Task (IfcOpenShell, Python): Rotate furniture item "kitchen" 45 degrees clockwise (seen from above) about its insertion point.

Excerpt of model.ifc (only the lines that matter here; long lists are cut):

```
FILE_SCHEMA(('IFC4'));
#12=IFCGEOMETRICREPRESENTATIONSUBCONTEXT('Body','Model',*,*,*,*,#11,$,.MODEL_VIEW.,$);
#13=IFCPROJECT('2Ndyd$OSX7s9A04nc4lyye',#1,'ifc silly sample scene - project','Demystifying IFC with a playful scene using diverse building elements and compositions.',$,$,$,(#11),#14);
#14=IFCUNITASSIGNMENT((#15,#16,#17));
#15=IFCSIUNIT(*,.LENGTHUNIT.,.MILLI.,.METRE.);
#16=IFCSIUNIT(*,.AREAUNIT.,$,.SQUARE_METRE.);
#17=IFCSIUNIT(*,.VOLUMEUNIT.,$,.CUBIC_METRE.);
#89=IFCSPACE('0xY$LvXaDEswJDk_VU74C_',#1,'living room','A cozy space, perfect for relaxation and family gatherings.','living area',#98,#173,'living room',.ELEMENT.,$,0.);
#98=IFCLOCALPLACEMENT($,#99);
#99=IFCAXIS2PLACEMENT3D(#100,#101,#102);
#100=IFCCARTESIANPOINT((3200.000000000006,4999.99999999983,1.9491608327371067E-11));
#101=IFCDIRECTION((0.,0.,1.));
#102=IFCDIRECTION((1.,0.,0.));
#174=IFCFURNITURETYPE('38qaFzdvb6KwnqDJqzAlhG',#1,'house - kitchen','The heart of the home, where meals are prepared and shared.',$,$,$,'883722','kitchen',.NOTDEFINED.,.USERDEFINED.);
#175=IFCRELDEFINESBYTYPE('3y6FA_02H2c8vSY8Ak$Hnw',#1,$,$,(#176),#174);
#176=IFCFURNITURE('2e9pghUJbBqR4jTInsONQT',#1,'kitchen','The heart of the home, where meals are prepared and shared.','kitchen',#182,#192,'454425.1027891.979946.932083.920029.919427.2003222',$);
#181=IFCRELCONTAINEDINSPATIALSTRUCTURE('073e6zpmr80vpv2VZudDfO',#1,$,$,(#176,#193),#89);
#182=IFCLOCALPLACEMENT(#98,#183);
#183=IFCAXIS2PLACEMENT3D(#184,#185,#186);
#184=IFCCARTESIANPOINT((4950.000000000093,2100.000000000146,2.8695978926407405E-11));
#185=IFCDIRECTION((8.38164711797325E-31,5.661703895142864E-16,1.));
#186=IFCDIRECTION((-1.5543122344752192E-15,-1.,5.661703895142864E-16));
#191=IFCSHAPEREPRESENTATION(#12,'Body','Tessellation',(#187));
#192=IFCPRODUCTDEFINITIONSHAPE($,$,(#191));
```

```python
import ifcopenshell
import ifcopenshell.api.geometry
import ifcopenshell.util.placement

model = ifcopenshell.open("model.ifc")

item = model.by_id(176)
matrix = ifcopenshell.util.placement.get_local_placement(item.ObjectPlacement)
matrix = matrix @ ifcopenshell.util.placement.rotation(-45, "Z")
ifcopenshell.api.geometry.edit_object_placement(model, product=item, matrix=matrix, is_si=False)

print(ifcopenshell.util.placement.get_local_placement(item.ObjectPlacement).round(3) + 0.0)

model.write("model-out.ifc")
```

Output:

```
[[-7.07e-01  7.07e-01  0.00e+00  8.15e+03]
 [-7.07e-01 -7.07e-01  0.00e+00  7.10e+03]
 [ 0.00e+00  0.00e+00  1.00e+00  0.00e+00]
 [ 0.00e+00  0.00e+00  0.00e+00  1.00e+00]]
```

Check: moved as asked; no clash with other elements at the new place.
